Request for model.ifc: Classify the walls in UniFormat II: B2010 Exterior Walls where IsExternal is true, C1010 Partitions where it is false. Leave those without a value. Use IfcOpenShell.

First a look at what the model holds.

```python
import ifcopenshell
import ifcopenshell.util.element

model = ifcopenshell.open("model.ifc")
print(model.schema)
print("classifications:", [c.Name for c in model.by_type("IfcClassification")])
values = [ifcopenshell.util.element.get_pset(e, "Pset_WallCommon", "IsExternal") for e in model.by_type("IfcWall")]
for value in (True, False, None):
    print("IsExternal", value, values.count(value))
```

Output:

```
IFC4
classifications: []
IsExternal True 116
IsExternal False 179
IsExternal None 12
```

```python
import ifcopenshell
import ifcopenshell.api.classification
import ifcopenshell.util.element

model = ifcopenshell.open("model.ifc")

system = ifcopenshell.api.classification.add_classification(model, classification="UniFormat II")

walls = model.by_type("IfcWall")
external = {e: ifcopenshell.util.element.get_pset(e, "Pset_WallCommon", "IsExternal") for e in walls}
for flag, code, name in ((True, "B2010", "Exterior Walls"), (False, "C1010", "Partitions")):
    products = [e for e in walls if external[e] is flag]
    ifcopenshell.api.classification.add_reference(
        model, products=products, classification=system, identification=code, name=name
    )
    print(code, len(products))

model.write("model_v2.ifc")
```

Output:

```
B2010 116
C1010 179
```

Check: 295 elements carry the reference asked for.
